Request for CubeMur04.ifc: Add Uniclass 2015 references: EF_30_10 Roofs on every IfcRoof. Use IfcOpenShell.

First a look at what the model holds.

```python
import ifcopenshell

model = ifcopenshell.open("CubeMur04.ifc")
print(model.schema)
print("classifications:", [c.Name for c in model.by_type("IfcClassification")])
for ifc_class in ("IfcDoor", "IfcRoof", "IfcStair", "IfcWall", "IfcWindow"):
    print(ifc_class, len(model.by_type(ifc_class)))
```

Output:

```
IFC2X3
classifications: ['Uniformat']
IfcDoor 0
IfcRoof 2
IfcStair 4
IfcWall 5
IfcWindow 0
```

```python
import ifcopenshell
import ifcopenshell.api.classification

model = ifcopenshell.open("CubeMur04.ifc")

# IFC2X3 requires Source and Edition and has no link from the project to the system.
system = model.create_entity("IfcClassification", Source="NBS", Edition="2015", Name="Uniclass 2015")

codes = {
    "IfcRoof": ("EF_30_10", "Roofs"),
}
for ifc_class, (code, name) in codes.items():
    products = model.by_type(ifc_class)
    ifcopenshell.api.classification.add_reference(
        model, products=products, classification=system, identification=code, name=name
    )
    print(code, len(products))

model.write("CubeMur04-out.ifc")
```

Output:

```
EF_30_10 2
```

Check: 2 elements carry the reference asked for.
